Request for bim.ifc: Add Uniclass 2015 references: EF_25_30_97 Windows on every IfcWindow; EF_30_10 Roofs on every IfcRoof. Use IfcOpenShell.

First a look at what the model holds.

```python
import ifcopenshell

model = ifcopenshell.open("bim.ifc")
print(model.schema)
print("classifications:", [c.Name for c in model.by_type("IfcClassification")])
for ifc_class in ("IfcDoor", "IfcRoof", "IfcStair", "IfcWall", "IfcWindow"):
    print(ifc_class, len(model.by_type(ifc_class)))
```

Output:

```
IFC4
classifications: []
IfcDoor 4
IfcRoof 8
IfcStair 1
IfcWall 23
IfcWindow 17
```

```python
import ifcopenshell
import ifcopenshell.api.classification

model = ifcopenshell.open("bim.ifc")

system = ifcopenshell.api.classification.add_classification(model, classification="Uniclass 2015")

codes = {
    "IfcWindow": ("EF_25_30_97", "Windows"),
    "IfcRoof": ("EF_30_10", "Roofs"),
}
for ifc_class, (code, name) in codes.items():
    products = model.by_type(ifc_class)
    ifcopenshell.api.classification.add_reference(
        model, products=products, classification=system, identification=code, name=name
    )
    print(code, len(products))

model.write("bim_edited.ifc")
```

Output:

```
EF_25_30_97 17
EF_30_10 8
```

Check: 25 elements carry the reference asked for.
